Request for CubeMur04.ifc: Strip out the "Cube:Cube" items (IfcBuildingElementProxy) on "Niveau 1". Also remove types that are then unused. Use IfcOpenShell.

First a look at what the model holds.

```python
import ifcopenshell
import ifcopenshell.util.element

model = ifcopenshell.open("CubeMur04.ifc")
print(model.schema)
storey = next(s for s in model.by_type("IfcBuildingStorey") if s.Name == "Niveau 1")
proxies = [e for e in ifcopenshell.util.element.get_decomposition(storey) if e.is_a("IfcBuildingElementProxy")]
seen = {}
for e in proxies:
    element_type = ifcopenshell.util.element.get_type(e)
    name = element_type.Name if element_type not in (None, e) else None
    seen[name] = seen.get(name, 0) + 1
for name, count in sorted(seen.items(), key=str):
    print(count, "x", name)
```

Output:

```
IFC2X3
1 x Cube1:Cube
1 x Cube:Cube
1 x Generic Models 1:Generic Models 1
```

```python
import ifcopenshell
import ifcopenshell.api.root
import ifcopenshell.util.element

model = ifcopenshell.open("CubeMur04.ifc")

storey = next(s for s in model.by_type("IfcBuildingStorey") if s.Name == "Niveau 1")
proxies = [e for e in ifcopenshell.util.element.get_decomposition(storey) if e.is_a("IfcBuildingElementProxy")]
targets = [e for e in proxies if (t := ifcopenshell.util.element.get_type(e)) not in (None, e) and t.Name == "Cube:Cube"]
types = {ifcopenshell.util.element.get_type(e) for e in targets} - {None, *targets}

for e in targets:
    ifcopenshell.api.root.remove_product(model, product=e)
print(len(targets), "removed")

unused = [t for t in types if not ifcopenshell.util.element.get_types(t)]
for t in unused:
    ifcopenshell.api.root.remove_product(model, product=t)
print(len(unused), "unused types removed")

model.write("CubeMur04-out.ifc")
```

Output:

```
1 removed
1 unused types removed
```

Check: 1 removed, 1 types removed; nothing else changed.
